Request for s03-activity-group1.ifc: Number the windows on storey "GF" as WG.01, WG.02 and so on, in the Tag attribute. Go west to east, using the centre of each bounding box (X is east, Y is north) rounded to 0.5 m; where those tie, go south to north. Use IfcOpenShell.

First a look at what the model holds.

```python
import ifcopenshell
import ifcopenshell.util.element
import ifcopenshell.util.placement

model = ifcopenshell.open("s03-activity-group1.ifc")
print(model.schema)
storey = next(s for s in model.by_type("IfcBuildingStorey") if s.Name == "GF")
windows = [e for e in ifcopenshell.util.element.get_decomposition(storey) if e.is_a("IfcWindow")]
for e in sorted(windows, key=lambda e: e.id()):
    origin = ifcopenshell.util.placement.get_local_placement(e.ObjectPlacement)[:3, 3]
    print(e.id(), e.Tag, e.Name, origin.round(2) + 0.0, sep=" | ")
```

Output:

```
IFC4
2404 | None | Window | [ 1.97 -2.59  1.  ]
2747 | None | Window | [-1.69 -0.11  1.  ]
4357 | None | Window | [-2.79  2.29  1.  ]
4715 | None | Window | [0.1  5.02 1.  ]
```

```python
import ifcopenshell
import ifcopenshell.geom
import ifcopenshell.util.element
import ifcopenshell.util.shape

model = ifcopenshell.open("s03-activity-group1.ifc")
settings = ifcopenshell.geom.settings()
settings.set("use-world-coords", True)


def centre(element):
    shape = ifcopenshell.geom.create_shape(settings, element)
    return ifcopenshell.util.shape.get_bbox_centroid(shape.geometry)


storey = next(s for s in model.by_type("IfcBuildingStorey") if s.Name == "GF")
windows = [e for e in ifcopenshell.util.element.get_decomposition(storey) if e.is_a("IfcWindow")]

# Insertion points can sit at a corner or the storey origin, so sort by the geometry (in metres).
centres = {e: centre(e) for e in windows}
windows.sort(key=lambda e: (round(centres[e][0] / 0.5), centres[e][1]))

for i, e in enumerate(windows, start=1):
    number = f"WG.{i:02d}"
    e.Tag = number
    print(e.id(), number)

model.write("s03-activity-group1-out.ifc")
```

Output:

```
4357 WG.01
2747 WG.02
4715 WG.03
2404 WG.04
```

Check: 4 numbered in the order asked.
